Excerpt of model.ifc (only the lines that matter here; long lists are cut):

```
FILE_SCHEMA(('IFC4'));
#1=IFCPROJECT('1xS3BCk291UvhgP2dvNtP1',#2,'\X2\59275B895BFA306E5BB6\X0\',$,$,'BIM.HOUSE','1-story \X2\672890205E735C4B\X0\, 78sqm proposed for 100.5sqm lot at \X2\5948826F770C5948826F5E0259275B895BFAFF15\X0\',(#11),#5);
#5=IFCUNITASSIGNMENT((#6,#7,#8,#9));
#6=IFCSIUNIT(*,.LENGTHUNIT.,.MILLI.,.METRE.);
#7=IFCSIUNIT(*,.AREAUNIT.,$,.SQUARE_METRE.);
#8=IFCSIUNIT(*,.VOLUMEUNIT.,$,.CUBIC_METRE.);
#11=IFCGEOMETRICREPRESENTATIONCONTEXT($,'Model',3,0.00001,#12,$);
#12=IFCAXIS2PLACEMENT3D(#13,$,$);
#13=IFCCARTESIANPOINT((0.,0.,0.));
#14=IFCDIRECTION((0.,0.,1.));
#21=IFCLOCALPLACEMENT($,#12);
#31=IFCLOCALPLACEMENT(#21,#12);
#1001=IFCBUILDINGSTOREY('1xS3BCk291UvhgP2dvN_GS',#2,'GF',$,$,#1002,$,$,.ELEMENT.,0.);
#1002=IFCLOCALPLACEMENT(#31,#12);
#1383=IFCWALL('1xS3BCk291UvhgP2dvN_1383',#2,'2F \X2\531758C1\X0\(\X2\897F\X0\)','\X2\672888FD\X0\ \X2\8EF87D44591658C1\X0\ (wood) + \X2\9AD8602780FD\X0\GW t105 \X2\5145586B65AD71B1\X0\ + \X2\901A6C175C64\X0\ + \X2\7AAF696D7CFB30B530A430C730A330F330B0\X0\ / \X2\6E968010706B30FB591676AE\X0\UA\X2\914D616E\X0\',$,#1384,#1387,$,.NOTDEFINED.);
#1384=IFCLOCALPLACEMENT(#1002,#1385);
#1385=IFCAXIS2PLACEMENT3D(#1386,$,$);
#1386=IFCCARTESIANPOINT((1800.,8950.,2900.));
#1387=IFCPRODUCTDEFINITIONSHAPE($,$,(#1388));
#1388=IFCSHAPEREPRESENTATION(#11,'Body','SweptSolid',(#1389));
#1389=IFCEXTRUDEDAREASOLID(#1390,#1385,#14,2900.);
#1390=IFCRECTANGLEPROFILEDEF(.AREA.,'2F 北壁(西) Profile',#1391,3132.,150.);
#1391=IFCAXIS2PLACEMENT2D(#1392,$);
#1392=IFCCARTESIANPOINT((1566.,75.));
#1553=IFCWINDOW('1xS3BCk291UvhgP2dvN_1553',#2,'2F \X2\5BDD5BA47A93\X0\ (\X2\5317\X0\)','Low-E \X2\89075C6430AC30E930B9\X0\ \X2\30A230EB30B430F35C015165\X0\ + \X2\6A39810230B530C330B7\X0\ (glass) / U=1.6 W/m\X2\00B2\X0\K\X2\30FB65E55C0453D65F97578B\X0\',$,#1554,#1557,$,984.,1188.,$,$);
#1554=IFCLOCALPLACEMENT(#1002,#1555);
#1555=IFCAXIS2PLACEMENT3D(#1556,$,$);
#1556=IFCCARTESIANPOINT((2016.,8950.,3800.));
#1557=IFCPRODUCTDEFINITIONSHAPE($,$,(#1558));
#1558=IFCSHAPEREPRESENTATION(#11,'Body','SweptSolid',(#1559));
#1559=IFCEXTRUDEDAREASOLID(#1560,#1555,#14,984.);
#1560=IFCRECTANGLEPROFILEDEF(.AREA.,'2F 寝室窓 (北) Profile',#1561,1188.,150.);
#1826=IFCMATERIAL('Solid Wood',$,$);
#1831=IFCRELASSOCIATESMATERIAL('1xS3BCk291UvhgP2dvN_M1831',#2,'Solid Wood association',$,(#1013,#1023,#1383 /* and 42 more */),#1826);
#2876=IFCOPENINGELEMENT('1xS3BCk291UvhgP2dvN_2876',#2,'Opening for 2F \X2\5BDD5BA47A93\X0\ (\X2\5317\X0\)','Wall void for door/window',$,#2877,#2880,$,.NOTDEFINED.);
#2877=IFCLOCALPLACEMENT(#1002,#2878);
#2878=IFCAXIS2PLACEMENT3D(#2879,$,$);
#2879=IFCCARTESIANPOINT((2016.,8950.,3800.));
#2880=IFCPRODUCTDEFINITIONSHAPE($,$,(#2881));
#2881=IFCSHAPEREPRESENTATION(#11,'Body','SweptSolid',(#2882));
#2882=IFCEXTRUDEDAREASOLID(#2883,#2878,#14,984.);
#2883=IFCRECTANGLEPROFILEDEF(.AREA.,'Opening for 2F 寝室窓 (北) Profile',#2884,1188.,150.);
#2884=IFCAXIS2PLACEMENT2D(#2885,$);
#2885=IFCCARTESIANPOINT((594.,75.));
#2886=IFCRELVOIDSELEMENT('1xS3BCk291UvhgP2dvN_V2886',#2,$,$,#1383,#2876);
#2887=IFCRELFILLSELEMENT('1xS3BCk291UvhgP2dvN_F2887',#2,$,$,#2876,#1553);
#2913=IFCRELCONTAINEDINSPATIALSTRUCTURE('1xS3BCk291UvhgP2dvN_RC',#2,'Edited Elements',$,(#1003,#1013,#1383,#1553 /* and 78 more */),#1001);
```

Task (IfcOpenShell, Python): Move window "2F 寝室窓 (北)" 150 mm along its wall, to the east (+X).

```python
import ifcopenshell
import ifcopenshell.api.geometry
import ifcopenshell.util.placement

model = ifcopenshell.open("model.ifc")

window = model.by_id(1553)
opening = window.FillsVoids[0].RelatingOpeningElement
wall = opening.VoidsElements[0].RelatingBuildingElement

wall_matrix = ifcopenshell.util.placement.get_local_placement(wall.ObjectPlacement)
shift = wall_matrix[:3, 0] * 150.0
before = ifcopenshell.util.placement.get_local_placement(window.ObjectPlacement)[:3, 3].copy()

# The window is not placed relative to its opening, so move both.
for product in (opening, window):
    matrix = ifcopenshell.util.placement.get_local_placement(product.ObjectPlacement)
    matrix[:3, 3] += shift
    ifcopenshell.api.geometry.edit_object_placement(model, product=product, matrix=matrix, is_si=False)

after = ifcopenshell.util.placement.get_local_placement(window.ObjectPlacement)[:3, 3]
print("window moved by", (after - before).round(3) + 0.0)

model.write("model_edited.ifc")
```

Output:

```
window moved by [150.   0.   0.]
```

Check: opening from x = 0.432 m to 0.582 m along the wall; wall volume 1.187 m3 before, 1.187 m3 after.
